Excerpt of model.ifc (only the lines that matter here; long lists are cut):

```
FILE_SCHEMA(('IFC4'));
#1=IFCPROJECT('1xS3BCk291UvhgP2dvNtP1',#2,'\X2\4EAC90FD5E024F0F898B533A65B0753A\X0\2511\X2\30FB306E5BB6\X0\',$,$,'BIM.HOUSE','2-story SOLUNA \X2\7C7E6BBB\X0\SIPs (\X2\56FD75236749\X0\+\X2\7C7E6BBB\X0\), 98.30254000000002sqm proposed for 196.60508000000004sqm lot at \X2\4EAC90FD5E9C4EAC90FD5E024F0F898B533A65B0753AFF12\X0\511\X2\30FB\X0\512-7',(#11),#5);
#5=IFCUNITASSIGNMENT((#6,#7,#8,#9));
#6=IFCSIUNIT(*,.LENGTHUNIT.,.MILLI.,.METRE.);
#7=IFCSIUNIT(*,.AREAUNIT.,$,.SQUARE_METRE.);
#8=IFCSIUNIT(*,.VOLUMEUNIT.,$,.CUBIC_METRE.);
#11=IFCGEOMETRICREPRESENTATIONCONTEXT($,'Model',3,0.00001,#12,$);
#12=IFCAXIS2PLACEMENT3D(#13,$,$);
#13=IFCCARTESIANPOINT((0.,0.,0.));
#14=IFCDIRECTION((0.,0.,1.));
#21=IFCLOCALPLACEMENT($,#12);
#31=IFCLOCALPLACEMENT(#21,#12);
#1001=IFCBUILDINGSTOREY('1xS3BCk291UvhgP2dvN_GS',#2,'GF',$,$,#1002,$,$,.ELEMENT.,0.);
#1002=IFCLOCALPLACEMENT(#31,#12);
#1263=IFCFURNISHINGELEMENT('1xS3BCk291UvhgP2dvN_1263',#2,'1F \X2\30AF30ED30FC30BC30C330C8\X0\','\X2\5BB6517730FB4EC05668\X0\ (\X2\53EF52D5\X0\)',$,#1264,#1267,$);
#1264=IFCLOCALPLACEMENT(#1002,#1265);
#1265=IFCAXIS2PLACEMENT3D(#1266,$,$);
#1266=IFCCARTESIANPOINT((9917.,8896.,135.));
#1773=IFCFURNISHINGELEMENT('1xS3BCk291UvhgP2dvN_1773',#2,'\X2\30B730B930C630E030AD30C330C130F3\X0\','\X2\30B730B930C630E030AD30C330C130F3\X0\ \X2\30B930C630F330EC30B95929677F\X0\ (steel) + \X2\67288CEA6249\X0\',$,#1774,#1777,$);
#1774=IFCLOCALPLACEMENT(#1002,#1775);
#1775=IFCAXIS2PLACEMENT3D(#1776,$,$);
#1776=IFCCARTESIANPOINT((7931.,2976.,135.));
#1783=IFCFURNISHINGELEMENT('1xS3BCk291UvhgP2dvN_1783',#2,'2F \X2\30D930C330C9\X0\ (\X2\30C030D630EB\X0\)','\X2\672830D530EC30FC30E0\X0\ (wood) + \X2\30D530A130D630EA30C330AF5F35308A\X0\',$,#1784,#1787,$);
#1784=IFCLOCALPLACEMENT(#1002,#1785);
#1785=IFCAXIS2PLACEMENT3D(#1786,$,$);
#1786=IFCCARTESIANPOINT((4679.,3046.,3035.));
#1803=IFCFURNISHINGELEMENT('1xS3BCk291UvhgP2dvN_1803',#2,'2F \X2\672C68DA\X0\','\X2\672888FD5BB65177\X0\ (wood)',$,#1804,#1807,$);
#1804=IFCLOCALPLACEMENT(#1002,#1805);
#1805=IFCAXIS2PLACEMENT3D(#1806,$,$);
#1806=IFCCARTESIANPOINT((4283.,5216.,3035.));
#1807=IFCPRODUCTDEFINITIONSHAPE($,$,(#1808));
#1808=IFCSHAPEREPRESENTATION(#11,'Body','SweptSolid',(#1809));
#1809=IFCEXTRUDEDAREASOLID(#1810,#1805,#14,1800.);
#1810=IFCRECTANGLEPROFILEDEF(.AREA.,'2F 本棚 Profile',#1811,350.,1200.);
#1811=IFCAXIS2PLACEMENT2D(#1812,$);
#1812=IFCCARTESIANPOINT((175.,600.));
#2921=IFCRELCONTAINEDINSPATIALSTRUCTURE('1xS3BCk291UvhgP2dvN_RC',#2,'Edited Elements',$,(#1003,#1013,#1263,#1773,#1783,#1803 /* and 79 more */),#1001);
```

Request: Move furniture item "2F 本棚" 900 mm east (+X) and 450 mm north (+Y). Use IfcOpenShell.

```python
import ifcopenshell
import ifcopenshell.api.geometry
import ifcopenshell.util.placement
import ifcopenshell.util.unit

model = ifcopenshell.open("model.ifc")
unit_scale = ifcopenshell.util.unit.calculate_unit_scale(model)

item = model.by_guid("1xS3BCk291UvhgP2dvN_1803")
matrix = ifcopenshell.util.placement.get_local_placement(item.ObjectPlacement)
matrix[0, 3] += 0.9 / unit_scale
matrix[1, 3] += 0.45 / unit_scale
ifcopenshell.api.geometry.edit_object_placement(model, product=item, matrix=matrix, is_si=False)

print(ifcopenshell.util.placement.get_local_placement(item.ObjectPlacement).round(3) + 0.0)

model.write("model_updated.ifc")
```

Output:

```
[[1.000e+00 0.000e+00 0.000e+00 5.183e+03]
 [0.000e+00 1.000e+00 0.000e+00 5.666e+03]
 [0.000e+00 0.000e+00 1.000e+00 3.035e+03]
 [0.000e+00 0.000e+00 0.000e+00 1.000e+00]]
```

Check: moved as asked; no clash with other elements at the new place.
